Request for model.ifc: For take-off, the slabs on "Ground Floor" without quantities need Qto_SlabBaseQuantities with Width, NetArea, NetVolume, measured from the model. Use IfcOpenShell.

First a look at what the model holds.

```python
import ifcopenshell
import ifcopenshell.util.element
import ifcopenshell.util.unit

model = ifcopenshell.open("model.ifc")
print(model.schema)
for unit_type in ("LENGTHUNIT", "AREAUNIT", "VOLUMEUNIT"):
    print(unit_type, ifcopenshell.util.unit.calculate_unit_scale(model, unit_type))
storey = next(s for s in model.by_type("IfcBuildingStorey") if s.Name == "Ground Floor")
slabs = [e for e in ifcopenshell.util.element.get_decomposition(storey) if e.is_a("IfcSlab")]
for e in sorted(slabs, key=lambda e: e.id()):
    print(e.id(), e.is_a(), e.Name, list(ifcopenshell.util.element.get_psets(e, qtos_only=True)), sep=" | ")
```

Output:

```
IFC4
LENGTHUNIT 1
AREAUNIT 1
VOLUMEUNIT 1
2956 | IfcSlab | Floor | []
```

```python
import ifcopenshell
import ifcopenshell.api.pset
import ifcopenshell.geom
import ifcopenshell.util.element
import ifcopenshell.util.shape
import ifcopenshell.util.unit

model = ifcopenshell.open("model.ifc")
unit_scale = ifcopenshell.util.unit.calculate_unit_scale(model)
area_scale = ifcopenshell.util.unit.calculate_unit_scale(model, "AREAUNIT")
volume_scale = ifcopenshell.util.unit.calculate_unit_scale(model, "VOLUMEUNIT")
settings = ifcopenshell.geom.settings()

storey = next(s for s in model.by_type("IfcBuildingStorey") if s.Name == "Ground Floor")
slabs = [e for e in ifcopenshell.util.element.get_decomposition(storey) if e.is_a("IfcSlab")]

for e in sorted(slabs, key=lambda e: e.id()):
    if ifcopenshell.util.element.get_psets(e, qtos_only=True, should_inherit=False):
        continue
    # Geometry comes back in metres, in the element's own axes.
    shape = ifcopenshell.geom.create_shape(settings, e)
    values = {
        "Width": ifcopenshell.util.shape.get_z(shape.geometry) / unit_scale,
        "NetArea": ifcopenshell.util.shape.get_footprint_area(shape.geometry) / area_scale,
        "NetVolume": ifcopenshell.util.shape.get_volume(shape.geometry) / volume_scale,
    }
    qto = ifcopenshell.api.pset.add_qto(model, product=e, name="Qto_SlabBaseQuantities")
    ifcopenshell.api.pset.edit_qto(model, qto=qto, properties=values)
    print(e.id(), {k: round(v, 3) for k, v in values.items()})

model.write("model_edited.ifc")
```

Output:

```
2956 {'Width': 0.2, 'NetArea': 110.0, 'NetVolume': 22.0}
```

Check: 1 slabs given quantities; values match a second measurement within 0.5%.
